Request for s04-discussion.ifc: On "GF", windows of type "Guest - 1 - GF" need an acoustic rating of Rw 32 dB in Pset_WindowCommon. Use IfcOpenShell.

First a look at what the model holds.

```python
import ifcopenshell
import ifcopenshell.util.element

model = ifcopenshell.open("s04-discussion.ifc")
print(model.schema)
storey = next(s for s in model.by_type("IfcBuildingStorey") if s.Name == "GF")
windows = [e for e in ifcopenshell.util.element.get_decomposition(storey) if e.is_a("IfcWindow")]
seen = {}
for e in windows:
    element_type = ifcopenshell.util.element.get_type(e)
    key = (element_type.Name if element_type != e and element_type else None, ifcopenshell.util.element.get_pset(e, "Pset_WindowCommon", "AcousticRating"))
    seen[key] = seen.get(key, 0) + 1
for (name, value), count in sorted(seen.items(), key=str):
    print(count, "x", name, "|", value)
```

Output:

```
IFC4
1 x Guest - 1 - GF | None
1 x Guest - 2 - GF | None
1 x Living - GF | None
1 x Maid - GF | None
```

```python
import ifcopenshell
import ifcopenshell.api.pset
import ifcopenshell.util.element

model = ifcopenshell.open("s04-discussion.ifc")

storey = next(s for s in model.by_type("IfcBuildingStorey") if s.Name == "GF")
windows = [e for e in ifcopenshell.util.element.get_decomposition(storey) if e.is_a("IfcWindow")]

count = 0
for e in windows:
    element_type = ifcopenshell.util.element.get_type(e)
    if element_type in (None, e) or element_type.Name != "Guest - 1 - GF":
        continue
    # add_pset returns the element's existing set when there is one.
    pset = ifcopenshell.api.pset.add_pset(model, product=e, name="Pset_WindowCommon")
    ifcopenshell.api.pset.edit_pset(model, pset=pset, properties={"AcousticRating": "Rw 32 dB"})
    count += 1

print(count, "windows updated")

model.write("s04-discussion_updated.ifc")
```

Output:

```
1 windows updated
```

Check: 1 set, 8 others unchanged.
